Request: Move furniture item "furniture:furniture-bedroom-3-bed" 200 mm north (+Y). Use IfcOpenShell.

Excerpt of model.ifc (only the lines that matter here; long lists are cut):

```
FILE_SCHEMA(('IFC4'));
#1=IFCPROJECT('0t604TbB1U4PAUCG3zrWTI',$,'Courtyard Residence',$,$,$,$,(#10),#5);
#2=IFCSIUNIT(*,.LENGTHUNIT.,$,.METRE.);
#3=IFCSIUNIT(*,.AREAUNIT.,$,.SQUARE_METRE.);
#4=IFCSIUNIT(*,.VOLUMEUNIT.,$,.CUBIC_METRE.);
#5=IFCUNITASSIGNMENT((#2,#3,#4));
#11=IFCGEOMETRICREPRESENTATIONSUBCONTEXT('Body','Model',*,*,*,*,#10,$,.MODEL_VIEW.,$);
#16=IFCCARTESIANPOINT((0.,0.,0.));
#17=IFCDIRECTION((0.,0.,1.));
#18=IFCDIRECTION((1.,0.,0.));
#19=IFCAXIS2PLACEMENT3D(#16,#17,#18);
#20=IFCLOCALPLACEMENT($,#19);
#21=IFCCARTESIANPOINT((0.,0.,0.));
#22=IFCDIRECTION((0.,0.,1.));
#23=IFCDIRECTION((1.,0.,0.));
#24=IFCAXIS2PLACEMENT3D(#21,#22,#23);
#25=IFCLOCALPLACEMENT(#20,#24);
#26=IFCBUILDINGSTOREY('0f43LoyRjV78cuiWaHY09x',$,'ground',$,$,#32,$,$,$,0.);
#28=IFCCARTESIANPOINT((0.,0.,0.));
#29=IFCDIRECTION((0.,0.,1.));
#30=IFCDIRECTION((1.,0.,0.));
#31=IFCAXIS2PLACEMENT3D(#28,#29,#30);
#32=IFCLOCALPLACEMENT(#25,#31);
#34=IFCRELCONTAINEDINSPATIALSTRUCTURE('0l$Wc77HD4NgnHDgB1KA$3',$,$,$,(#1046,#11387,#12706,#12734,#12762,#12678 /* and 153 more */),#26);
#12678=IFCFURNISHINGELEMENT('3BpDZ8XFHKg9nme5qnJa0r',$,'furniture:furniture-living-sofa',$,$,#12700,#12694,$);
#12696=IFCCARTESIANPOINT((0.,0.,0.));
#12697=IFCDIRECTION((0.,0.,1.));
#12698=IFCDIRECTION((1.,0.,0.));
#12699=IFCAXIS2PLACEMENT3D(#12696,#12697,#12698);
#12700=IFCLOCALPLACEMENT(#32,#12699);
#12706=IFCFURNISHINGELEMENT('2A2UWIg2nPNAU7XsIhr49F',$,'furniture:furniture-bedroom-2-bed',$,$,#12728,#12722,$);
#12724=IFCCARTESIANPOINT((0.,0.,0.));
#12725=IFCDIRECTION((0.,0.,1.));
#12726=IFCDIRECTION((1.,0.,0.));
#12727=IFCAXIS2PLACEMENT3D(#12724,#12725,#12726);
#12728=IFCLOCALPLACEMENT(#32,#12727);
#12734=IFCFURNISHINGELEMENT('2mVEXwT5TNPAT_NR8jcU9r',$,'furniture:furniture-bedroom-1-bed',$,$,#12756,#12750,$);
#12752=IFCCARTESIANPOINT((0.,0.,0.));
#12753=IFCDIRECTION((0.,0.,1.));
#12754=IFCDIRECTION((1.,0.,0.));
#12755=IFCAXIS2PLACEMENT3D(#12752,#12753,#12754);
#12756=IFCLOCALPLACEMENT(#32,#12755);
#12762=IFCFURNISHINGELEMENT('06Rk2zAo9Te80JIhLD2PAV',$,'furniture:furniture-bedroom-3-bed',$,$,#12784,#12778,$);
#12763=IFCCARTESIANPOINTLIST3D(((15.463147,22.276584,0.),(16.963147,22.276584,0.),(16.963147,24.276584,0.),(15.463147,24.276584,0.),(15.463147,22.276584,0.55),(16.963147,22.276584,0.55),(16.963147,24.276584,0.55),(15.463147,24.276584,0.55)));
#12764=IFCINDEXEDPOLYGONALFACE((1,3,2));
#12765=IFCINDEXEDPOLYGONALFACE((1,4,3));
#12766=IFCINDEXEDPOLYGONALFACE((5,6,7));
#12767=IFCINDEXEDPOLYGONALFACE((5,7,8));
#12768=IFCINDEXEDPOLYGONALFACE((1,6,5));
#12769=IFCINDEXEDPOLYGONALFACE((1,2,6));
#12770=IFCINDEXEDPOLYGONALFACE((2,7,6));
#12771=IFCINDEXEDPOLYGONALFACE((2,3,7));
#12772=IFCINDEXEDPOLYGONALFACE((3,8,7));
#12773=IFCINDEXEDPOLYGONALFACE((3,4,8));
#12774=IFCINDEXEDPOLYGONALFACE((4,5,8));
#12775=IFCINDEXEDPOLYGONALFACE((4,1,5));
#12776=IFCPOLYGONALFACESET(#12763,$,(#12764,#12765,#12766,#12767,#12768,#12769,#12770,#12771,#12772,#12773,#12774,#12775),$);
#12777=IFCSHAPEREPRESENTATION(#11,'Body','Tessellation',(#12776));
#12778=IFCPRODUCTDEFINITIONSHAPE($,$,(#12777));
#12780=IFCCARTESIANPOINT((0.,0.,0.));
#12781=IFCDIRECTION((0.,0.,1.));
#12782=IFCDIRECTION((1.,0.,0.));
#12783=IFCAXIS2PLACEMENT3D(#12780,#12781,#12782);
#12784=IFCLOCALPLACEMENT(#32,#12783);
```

```python
import ifcopenshell
import ifcopenshell.api.geometry
import ifcopenshell.util.placement

model = ifcopenshell.open("model.ifc")

item = model.by_id(12762)
matrix = ifcopenshell.util.placement.get_local_placement(item.ObjectPlacement)
matrix[1, 3] += 0.2
ifcopenshell.api.geometry.edit_object_placement(model, product=item, matrix=matrix, is_si=False)

print(ifcopenshell.util.placement.get_local_placement(item.ObjectPlacement).round(3) + 0.0)

model.write("model_edited.ifc")
```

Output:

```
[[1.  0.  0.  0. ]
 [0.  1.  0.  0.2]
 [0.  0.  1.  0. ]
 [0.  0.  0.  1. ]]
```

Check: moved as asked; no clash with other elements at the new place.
